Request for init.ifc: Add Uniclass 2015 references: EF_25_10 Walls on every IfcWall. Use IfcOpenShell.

First a look at what the model holds.

```python
import ifcopenshell

model = ifcopenshell.open("init.ifc")
print(model.schema)
print("classifications:", [c.Name for c in model.by_type("IfcClassification")])
for ifc_class in ("IfcDoor", "IfcRoof", "IfcStair", "IfcWall", "IfcWindow"):
    print(ifc_class, len(model.by_type(ifc_class)))
```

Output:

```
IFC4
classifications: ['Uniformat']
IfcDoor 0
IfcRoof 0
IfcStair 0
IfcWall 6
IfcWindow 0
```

```python
import ifcopenshell
import ifcopenshell.api.classification

model = ifcopenshell.open("init.ifc")

system = ifcopenshell.api.classification.add_classification(model, classification="Uniclass 2015")

codes = {
    "IfcWall": ("EF_25_10", "Walls"),
}
for ifc_class, (code, name) in codes.items():
    products = model.by_type(ifc_class)
    ifcopenshell.api.classification.add_reference(
        model, products=products, classification=system, identification=code, name=name
    )
    print(code, len(products))

model.write("init_v2.ifc")
```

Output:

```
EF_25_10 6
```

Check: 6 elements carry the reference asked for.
